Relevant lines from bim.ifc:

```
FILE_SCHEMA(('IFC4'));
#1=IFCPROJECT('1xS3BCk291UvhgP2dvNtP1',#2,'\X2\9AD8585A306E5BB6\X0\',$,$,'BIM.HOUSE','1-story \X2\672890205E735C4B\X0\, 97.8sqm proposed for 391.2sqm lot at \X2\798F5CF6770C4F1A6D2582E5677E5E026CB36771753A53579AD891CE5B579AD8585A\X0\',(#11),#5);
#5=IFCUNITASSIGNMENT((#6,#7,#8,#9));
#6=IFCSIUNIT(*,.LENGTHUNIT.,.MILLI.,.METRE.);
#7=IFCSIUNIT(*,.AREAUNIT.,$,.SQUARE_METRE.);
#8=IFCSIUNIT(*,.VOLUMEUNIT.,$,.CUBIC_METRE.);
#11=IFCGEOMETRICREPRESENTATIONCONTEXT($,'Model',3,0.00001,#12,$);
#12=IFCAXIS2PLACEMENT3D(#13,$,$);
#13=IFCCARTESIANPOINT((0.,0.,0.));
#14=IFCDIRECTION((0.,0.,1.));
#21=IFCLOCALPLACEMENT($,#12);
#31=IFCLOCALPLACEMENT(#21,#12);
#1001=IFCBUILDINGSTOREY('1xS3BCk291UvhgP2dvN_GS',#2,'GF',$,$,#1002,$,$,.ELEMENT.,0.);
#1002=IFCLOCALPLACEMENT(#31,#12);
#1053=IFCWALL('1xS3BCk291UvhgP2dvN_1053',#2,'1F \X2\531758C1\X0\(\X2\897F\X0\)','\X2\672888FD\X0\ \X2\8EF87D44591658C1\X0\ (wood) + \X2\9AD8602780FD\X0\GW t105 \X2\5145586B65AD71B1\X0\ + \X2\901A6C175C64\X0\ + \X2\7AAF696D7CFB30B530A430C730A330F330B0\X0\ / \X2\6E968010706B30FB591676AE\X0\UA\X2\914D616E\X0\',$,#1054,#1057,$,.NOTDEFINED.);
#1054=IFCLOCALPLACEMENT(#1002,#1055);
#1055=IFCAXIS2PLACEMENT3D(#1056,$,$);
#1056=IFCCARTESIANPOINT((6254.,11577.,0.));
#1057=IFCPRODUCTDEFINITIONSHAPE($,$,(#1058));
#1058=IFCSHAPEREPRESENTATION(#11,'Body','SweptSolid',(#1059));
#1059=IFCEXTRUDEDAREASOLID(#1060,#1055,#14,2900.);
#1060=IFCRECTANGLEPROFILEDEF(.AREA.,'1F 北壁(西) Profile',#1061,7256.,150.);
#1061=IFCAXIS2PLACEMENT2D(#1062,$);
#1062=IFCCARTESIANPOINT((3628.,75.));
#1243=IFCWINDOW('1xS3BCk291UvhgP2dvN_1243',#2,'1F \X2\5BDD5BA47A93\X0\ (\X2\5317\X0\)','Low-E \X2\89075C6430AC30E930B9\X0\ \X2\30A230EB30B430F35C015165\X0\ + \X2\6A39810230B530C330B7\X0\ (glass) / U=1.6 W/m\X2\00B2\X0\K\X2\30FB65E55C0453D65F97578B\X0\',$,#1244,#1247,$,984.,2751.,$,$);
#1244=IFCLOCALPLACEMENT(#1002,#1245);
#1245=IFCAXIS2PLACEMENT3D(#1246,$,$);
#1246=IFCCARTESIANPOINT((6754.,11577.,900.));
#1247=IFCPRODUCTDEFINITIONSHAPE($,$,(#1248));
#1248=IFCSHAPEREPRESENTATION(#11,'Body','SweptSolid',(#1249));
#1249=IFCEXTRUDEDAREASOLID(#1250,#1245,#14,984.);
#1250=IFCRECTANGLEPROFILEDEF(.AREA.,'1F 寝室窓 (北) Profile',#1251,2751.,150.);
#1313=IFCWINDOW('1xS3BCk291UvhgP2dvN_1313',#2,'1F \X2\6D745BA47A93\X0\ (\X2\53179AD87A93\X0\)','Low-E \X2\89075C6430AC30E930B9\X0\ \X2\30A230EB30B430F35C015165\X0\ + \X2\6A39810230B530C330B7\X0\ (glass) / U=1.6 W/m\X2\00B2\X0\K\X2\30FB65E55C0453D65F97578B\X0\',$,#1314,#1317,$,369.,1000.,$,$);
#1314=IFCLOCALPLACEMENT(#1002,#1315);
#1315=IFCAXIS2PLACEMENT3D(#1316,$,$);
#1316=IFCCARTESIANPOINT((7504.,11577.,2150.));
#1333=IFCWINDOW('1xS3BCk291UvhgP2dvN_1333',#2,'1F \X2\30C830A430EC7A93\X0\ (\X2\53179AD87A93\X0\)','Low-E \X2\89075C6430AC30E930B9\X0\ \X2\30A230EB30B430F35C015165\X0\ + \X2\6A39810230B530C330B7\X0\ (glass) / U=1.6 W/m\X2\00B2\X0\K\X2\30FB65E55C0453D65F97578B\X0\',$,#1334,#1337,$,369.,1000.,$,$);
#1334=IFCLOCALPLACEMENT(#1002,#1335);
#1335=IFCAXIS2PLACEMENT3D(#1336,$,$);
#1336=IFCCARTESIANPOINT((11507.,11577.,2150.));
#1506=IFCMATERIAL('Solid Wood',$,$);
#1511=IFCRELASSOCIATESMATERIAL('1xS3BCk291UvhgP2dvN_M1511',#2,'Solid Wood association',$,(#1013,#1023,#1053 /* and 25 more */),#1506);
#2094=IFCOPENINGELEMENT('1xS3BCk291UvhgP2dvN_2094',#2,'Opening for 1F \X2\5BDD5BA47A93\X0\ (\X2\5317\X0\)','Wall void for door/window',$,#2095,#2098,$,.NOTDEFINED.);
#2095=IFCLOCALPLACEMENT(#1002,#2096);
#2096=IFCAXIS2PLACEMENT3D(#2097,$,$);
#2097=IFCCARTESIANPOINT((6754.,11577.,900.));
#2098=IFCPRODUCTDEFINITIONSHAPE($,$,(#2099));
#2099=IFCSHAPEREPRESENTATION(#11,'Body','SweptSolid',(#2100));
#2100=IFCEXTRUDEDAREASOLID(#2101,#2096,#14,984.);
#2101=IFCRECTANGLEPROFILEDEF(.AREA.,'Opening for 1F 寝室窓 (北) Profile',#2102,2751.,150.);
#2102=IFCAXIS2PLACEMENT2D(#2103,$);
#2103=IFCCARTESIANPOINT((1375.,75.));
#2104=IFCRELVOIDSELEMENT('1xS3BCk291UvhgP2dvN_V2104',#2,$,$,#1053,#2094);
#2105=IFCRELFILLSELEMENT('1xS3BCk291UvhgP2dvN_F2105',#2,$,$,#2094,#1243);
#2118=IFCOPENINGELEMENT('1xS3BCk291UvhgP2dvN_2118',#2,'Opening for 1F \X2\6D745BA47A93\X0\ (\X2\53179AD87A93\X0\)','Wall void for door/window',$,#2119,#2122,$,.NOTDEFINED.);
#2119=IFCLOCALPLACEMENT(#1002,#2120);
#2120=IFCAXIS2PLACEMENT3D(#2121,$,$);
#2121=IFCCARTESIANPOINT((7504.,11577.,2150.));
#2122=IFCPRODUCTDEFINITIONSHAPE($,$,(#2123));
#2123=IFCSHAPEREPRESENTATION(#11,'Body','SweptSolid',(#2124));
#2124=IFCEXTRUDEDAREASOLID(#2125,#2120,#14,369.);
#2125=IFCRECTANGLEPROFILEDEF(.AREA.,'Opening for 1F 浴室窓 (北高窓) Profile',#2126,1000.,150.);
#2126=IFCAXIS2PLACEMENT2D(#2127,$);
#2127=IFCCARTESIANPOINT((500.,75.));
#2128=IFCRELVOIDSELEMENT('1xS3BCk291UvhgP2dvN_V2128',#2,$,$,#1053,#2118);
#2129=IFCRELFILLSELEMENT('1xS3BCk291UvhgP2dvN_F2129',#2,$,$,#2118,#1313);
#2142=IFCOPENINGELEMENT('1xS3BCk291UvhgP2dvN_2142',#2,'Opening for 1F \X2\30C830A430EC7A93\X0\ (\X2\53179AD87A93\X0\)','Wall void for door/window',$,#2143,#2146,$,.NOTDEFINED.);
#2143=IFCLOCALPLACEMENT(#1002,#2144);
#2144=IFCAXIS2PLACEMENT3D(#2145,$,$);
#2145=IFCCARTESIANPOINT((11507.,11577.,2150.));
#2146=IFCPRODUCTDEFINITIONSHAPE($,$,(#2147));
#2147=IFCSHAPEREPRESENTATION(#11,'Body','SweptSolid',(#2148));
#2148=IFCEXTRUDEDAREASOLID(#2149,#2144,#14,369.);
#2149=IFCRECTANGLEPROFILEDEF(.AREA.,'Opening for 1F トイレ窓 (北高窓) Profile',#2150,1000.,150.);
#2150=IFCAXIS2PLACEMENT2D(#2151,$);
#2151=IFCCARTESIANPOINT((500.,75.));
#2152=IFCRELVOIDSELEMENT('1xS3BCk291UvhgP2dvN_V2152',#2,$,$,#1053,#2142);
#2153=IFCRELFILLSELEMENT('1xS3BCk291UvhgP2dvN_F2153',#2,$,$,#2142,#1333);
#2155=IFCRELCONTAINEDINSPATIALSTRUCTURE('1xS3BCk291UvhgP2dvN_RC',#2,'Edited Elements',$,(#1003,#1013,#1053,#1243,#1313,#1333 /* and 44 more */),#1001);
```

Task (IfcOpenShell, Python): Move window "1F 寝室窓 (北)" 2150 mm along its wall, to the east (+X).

```python
import ifcopenshell
import ifcopenshell.api.geometry
import ifcopenshell.util.placement

model = ifcopenshell.open("bim.ifc")

window = model.by_guid("1xS3BCk291UvhgP2dvN_1243")
opening = window.FillsVoids[0].RelatingOpeningElement
wall = opening.VoidsElements[0].RelatingBuildingElement

wall_matrix = ifcopenshell.util.placement.get_local_placement(wall.ObjectPlacement)
shift = wall_matrix[:3, 0] * 2150.0
before = ifcopenshell.util.placement.get_local_placement(window.ObjectPlacement)[:3, 3].copy()

# The window is not placed relative to its opening, so move both.
for product in (opening, window):
    matrix = ifcopenshell.util.placement.get_local_placement(product.ObjectPlacement)
    matrix[:3, 3] += shift
    ifcopenshell.api.geometry.edit_object_placement(model, product=product, matrix=matrix, is_si=False)

after = ifcopenshell.util.placement.get_local_placement(window.ObjectPlacement)[:3, 3]
print("window moved by", (after - before).round(3) + 0.0)

model.write("bim-out.ifc")
```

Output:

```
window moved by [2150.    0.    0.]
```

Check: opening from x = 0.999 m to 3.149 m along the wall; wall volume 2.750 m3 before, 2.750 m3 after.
